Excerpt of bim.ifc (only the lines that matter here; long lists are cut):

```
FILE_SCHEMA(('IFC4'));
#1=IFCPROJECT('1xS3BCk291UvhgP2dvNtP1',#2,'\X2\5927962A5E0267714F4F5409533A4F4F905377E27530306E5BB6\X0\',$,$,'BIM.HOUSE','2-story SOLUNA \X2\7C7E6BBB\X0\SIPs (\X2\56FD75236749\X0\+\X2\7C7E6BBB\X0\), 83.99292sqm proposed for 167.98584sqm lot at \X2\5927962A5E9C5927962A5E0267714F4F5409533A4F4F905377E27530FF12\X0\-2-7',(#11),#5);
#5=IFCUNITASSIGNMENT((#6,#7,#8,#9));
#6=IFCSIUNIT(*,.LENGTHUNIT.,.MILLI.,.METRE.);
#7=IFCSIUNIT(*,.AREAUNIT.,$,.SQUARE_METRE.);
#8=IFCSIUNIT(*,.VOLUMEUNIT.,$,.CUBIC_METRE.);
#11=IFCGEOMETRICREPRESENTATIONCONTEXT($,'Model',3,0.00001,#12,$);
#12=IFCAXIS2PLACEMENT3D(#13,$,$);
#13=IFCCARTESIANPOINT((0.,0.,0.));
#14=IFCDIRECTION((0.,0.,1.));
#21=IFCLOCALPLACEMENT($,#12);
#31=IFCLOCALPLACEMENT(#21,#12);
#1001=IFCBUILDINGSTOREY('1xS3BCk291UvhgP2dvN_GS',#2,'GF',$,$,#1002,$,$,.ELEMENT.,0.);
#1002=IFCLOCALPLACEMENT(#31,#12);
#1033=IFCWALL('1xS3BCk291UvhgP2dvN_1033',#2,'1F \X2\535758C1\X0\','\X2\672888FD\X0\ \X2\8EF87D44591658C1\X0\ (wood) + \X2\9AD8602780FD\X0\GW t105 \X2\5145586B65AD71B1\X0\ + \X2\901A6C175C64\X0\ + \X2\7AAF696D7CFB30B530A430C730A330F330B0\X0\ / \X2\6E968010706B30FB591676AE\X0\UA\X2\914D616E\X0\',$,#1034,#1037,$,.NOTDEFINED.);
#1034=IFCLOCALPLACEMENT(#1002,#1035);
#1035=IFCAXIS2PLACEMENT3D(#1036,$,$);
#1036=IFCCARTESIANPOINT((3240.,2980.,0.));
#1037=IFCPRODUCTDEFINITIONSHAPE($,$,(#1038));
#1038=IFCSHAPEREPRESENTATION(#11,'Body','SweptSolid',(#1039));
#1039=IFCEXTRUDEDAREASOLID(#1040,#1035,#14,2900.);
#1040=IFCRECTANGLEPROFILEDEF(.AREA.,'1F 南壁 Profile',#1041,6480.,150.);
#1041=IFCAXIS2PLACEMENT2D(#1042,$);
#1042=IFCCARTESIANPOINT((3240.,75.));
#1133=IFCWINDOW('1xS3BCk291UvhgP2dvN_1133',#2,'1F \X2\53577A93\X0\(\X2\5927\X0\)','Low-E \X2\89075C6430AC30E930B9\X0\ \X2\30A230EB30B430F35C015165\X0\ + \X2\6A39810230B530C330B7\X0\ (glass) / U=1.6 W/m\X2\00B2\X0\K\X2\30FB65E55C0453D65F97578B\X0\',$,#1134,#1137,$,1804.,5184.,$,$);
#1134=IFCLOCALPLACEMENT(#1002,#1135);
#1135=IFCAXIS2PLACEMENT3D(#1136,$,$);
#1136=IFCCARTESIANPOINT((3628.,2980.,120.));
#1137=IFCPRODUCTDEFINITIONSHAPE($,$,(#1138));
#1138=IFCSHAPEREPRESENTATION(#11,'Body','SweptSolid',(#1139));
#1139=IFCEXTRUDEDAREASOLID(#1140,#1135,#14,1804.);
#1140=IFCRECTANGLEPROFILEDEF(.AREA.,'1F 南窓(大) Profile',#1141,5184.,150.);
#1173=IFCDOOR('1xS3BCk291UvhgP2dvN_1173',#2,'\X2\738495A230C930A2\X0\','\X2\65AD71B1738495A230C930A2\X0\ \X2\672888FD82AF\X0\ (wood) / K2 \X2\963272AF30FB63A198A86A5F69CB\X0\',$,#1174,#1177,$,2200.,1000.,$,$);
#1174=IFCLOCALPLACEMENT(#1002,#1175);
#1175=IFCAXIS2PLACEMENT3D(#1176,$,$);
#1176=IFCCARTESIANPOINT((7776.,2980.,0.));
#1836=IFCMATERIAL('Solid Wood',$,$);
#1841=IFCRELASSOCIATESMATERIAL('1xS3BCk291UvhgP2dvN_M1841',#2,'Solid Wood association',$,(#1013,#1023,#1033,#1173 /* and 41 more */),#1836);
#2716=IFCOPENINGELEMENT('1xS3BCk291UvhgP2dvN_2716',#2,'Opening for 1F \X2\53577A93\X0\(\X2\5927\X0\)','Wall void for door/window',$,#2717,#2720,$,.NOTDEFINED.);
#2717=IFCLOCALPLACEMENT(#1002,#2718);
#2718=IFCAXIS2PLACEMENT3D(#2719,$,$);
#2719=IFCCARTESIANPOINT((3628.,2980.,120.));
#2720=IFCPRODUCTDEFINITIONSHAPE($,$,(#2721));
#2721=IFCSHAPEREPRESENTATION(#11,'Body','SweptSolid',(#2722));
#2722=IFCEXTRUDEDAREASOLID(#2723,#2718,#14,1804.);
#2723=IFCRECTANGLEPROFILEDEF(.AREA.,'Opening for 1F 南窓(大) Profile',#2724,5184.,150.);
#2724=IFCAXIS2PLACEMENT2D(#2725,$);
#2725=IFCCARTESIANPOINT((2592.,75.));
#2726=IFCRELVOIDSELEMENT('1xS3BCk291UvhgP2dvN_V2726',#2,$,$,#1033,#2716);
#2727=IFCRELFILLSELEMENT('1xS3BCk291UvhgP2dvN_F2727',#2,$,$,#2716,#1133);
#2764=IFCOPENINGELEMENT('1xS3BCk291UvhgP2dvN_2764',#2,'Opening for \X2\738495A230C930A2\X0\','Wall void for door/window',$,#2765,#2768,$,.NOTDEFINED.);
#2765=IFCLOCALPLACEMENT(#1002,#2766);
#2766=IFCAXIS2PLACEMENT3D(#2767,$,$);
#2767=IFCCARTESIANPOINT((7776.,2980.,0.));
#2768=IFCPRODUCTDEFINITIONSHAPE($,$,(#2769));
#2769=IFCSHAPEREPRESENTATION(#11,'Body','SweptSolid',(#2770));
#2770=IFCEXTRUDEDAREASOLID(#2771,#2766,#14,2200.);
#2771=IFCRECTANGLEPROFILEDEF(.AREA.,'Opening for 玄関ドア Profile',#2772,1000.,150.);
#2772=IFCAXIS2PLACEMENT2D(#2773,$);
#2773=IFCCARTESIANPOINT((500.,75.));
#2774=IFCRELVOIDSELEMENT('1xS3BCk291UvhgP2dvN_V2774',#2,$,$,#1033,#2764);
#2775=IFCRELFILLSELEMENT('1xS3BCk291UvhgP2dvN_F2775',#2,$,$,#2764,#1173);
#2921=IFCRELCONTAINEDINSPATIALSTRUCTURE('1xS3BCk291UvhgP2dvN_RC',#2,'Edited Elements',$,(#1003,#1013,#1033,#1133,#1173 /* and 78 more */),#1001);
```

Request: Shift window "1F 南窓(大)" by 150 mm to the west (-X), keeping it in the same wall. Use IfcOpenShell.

```python
import ifcopenshell
import ifcopenshell.api.geometry
import ifcopenshell.util.placement
import ifcopenshell.util.unit

model = ifcopenshell.open("bim.ifc")
unit_scale = ifcopenshell.util.unit.calculate_unit_scale(model)

window = model.by_id(1133)
opening = window.FillsVoids[0].RelatingOpeningElement
wall = opening.VoidsElements[0].RelatingBuildingElement

wall_matrix = ifcopenshell.util.placement.get_local_placement(wall.ObjectPlacement)
shift = wall_matrix[:3, 0] * -0.15 / unit_scale
before = ifcopenshell.util.placement.get_local_placement(window.ObjectPlacement)[:3, 3].copy()

# The window is not placed relative to its opening, so move both.
for product in (opening, window):
    matrix = ifcopenshell.util.placement.get_local_placement(product.ObjectPlacement)
    matrix[:3, 3] += shift
    ifcopenshell.api.geometry.edit_object_placement(model, product=product, matrix=matrix, is_si=False)

after = ifcopenshell.util.placement.get_local_placement(window.ObjectPlacement)[:3, 3]
print("window moved by", (after - before).round(3) + 0.0)

model.write("bim_v2.ifc")
```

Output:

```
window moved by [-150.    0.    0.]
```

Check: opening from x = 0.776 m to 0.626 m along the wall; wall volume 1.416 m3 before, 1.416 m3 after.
